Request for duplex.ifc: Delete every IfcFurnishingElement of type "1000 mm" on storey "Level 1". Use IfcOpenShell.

First a look at what the model holds.

```python
import ifcopenshell
import ifcopenshell.util.element

model = ifcopenshell.open("duplex.ifc")
print(model.schema)
storey = next(s for s in model.by_type("IfcBuildingStorey") if s.Name == "Level 1")
furniture = [e for e in ifcopenshell.util.element.get_decomposition(storey) if e.is_a("IfcFurnishingElement")]
seen = {}
for e in furniture:
    element_type = ifcopenshell.util.element.get_type(e)
    name = element_type.Name if element_type not in (None, e) else None
    seen[name] = seen.get(name, 0) + 1
for name, count in sorted(seen.items(), key=str):
    print(count, "x", name)
```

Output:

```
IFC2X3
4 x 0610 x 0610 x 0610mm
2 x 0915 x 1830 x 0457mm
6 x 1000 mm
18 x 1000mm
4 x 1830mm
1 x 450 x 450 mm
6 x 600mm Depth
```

```python
import ifcopenshell
import ifcopenshell.api.root
import ifcopenshell.util.element

model = ifcopenshell.open("duplex.ifc")

storey = next(s for s in model.by_type("IfcBuildingStorey") if s.Name == "Level 1")
furniture = [e for e in ifcopenshell.util.element.get_decomposition(storey) if e.is_a("IfcFurnishingElement")]
targets = [e for e in furniture if (t := ifcopenshell.util.element.get_type(e)) not in (None, e) and t.Name == "1000 mm"]

for e in targets:
    ifcopenshell.api.root.remove_product(model, product=e)
print(len(targets), "removed")

model.write("duplex_v2.ifc")
```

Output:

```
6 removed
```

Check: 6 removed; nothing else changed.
